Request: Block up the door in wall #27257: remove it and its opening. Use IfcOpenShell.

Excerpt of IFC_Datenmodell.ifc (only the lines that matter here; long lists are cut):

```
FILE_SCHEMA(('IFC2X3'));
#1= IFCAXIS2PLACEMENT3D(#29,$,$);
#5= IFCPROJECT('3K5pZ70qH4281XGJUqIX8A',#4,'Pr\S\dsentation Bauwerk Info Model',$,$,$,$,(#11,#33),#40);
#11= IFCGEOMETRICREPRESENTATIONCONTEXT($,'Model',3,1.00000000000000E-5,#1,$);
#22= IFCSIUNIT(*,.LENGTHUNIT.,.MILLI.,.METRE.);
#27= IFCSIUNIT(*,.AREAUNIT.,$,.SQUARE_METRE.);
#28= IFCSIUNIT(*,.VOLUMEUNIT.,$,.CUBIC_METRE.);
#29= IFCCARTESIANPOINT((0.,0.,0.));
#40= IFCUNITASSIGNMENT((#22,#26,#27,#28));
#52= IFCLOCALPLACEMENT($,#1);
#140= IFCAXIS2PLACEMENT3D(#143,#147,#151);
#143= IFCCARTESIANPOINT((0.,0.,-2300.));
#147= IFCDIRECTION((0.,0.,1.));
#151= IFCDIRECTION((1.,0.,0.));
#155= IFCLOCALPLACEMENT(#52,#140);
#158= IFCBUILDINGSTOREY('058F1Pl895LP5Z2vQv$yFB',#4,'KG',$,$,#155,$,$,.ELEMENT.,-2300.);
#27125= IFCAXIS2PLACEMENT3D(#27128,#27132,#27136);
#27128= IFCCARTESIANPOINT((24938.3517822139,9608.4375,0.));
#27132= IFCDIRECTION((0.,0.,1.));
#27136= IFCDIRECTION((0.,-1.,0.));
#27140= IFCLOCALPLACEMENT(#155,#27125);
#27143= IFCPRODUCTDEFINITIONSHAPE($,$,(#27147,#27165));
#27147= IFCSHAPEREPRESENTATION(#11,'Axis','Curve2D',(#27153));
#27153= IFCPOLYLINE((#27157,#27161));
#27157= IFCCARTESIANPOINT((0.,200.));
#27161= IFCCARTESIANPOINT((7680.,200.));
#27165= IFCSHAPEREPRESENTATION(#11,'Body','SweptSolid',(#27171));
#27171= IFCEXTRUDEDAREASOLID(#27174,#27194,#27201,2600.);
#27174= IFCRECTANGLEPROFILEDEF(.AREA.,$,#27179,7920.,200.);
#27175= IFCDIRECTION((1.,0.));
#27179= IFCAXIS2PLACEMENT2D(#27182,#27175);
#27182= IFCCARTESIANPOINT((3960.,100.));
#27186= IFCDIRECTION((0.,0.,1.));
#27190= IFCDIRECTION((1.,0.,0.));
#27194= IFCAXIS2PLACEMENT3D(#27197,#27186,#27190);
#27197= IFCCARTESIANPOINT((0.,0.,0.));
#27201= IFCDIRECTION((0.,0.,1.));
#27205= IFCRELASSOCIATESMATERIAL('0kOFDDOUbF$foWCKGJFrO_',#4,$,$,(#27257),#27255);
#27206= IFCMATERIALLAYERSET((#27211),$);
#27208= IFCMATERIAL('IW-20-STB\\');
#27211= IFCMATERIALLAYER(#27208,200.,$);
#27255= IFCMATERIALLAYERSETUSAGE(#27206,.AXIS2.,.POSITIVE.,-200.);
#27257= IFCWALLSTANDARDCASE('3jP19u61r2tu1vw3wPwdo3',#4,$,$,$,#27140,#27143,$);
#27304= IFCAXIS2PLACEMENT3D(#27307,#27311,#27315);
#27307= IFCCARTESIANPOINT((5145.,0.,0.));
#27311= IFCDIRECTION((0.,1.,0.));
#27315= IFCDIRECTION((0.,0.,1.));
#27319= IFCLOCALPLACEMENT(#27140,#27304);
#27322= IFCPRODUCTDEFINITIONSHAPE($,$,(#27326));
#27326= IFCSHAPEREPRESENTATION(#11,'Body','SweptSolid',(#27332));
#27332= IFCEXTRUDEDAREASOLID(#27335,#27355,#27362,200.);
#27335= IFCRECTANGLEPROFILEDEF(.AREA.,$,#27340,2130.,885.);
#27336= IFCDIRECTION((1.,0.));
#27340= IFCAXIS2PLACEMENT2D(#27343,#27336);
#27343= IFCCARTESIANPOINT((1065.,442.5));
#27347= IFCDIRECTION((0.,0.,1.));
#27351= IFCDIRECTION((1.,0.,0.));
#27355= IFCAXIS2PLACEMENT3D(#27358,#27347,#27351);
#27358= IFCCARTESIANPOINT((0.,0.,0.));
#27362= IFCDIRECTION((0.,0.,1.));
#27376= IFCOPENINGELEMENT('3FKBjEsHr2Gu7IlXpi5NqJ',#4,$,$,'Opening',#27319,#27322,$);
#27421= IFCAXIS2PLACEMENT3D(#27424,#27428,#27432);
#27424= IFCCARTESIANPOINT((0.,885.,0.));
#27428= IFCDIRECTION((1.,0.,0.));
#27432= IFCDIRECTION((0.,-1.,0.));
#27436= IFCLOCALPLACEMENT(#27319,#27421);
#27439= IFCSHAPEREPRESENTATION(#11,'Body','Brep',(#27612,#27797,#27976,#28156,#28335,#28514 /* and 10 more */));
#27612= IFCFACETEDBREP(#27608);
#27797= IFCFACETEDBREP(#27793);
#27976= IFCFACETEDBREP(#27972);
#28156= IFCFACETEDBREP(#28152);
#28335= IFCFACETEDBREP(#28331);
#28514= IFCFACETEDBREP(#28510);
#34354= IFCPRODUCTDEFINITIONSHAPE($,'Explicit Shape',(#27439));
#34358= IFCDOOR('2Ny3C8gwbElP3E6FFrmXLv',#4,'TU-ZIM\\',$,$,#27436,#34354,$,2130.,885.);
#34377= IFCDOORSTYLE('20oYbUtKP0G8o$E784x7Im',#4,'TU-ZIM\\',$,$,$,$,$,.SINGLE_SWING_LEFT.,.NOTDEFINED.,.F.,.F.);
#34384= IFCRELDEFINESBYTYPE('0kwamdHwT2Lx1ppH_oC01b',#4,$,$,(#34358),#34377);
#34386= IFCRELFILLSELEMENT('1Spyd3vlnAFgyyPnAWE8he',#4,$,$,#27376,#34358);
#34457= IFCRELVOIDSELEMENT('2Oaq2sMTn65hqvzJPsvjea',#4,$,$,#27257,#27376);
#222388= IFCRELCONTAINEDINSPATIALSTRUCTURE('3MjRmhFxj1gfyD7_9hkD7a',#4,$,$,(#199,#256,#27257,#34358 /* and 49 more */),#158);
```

```python
import ifcopenshell
import ifcopenshell.api.feature
import ifcopenshell.api.root
import ifcopenshell.geom
import ifcopenshell.util.shape

model = ifcopenshell.open("IFC_Datenmodell.ifc")
settings = ifcopenshell.geom.settings()


def volume(element):
    """Net volume in cubic metres, openings subtracted."""
    shape = ifcopenshell.geom.create_shape(settings, element)
    return ifcopenshell.util.shape.get_volume(shape.geometry)


door = model.by_id(34358)
opening = door.FillsVoids[0].RelatingOpeningElement
wall = opening.VoidsElements[0].RelatingBuildingElement
before = volume(wall)

ifcopenshell.api.root.remove_product(model, product=door)
ifcopenshell.api.feature.remove_feature(model, feature=opening)

after = volume(wall)

print(f"wall volume {before:.3f} -> {after:.3f} m3")

model.write("IFC_Datenmodell-out.ifc")
```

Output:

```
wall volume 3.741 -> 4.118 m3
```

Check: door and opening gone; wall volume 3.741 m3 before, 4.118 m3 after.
